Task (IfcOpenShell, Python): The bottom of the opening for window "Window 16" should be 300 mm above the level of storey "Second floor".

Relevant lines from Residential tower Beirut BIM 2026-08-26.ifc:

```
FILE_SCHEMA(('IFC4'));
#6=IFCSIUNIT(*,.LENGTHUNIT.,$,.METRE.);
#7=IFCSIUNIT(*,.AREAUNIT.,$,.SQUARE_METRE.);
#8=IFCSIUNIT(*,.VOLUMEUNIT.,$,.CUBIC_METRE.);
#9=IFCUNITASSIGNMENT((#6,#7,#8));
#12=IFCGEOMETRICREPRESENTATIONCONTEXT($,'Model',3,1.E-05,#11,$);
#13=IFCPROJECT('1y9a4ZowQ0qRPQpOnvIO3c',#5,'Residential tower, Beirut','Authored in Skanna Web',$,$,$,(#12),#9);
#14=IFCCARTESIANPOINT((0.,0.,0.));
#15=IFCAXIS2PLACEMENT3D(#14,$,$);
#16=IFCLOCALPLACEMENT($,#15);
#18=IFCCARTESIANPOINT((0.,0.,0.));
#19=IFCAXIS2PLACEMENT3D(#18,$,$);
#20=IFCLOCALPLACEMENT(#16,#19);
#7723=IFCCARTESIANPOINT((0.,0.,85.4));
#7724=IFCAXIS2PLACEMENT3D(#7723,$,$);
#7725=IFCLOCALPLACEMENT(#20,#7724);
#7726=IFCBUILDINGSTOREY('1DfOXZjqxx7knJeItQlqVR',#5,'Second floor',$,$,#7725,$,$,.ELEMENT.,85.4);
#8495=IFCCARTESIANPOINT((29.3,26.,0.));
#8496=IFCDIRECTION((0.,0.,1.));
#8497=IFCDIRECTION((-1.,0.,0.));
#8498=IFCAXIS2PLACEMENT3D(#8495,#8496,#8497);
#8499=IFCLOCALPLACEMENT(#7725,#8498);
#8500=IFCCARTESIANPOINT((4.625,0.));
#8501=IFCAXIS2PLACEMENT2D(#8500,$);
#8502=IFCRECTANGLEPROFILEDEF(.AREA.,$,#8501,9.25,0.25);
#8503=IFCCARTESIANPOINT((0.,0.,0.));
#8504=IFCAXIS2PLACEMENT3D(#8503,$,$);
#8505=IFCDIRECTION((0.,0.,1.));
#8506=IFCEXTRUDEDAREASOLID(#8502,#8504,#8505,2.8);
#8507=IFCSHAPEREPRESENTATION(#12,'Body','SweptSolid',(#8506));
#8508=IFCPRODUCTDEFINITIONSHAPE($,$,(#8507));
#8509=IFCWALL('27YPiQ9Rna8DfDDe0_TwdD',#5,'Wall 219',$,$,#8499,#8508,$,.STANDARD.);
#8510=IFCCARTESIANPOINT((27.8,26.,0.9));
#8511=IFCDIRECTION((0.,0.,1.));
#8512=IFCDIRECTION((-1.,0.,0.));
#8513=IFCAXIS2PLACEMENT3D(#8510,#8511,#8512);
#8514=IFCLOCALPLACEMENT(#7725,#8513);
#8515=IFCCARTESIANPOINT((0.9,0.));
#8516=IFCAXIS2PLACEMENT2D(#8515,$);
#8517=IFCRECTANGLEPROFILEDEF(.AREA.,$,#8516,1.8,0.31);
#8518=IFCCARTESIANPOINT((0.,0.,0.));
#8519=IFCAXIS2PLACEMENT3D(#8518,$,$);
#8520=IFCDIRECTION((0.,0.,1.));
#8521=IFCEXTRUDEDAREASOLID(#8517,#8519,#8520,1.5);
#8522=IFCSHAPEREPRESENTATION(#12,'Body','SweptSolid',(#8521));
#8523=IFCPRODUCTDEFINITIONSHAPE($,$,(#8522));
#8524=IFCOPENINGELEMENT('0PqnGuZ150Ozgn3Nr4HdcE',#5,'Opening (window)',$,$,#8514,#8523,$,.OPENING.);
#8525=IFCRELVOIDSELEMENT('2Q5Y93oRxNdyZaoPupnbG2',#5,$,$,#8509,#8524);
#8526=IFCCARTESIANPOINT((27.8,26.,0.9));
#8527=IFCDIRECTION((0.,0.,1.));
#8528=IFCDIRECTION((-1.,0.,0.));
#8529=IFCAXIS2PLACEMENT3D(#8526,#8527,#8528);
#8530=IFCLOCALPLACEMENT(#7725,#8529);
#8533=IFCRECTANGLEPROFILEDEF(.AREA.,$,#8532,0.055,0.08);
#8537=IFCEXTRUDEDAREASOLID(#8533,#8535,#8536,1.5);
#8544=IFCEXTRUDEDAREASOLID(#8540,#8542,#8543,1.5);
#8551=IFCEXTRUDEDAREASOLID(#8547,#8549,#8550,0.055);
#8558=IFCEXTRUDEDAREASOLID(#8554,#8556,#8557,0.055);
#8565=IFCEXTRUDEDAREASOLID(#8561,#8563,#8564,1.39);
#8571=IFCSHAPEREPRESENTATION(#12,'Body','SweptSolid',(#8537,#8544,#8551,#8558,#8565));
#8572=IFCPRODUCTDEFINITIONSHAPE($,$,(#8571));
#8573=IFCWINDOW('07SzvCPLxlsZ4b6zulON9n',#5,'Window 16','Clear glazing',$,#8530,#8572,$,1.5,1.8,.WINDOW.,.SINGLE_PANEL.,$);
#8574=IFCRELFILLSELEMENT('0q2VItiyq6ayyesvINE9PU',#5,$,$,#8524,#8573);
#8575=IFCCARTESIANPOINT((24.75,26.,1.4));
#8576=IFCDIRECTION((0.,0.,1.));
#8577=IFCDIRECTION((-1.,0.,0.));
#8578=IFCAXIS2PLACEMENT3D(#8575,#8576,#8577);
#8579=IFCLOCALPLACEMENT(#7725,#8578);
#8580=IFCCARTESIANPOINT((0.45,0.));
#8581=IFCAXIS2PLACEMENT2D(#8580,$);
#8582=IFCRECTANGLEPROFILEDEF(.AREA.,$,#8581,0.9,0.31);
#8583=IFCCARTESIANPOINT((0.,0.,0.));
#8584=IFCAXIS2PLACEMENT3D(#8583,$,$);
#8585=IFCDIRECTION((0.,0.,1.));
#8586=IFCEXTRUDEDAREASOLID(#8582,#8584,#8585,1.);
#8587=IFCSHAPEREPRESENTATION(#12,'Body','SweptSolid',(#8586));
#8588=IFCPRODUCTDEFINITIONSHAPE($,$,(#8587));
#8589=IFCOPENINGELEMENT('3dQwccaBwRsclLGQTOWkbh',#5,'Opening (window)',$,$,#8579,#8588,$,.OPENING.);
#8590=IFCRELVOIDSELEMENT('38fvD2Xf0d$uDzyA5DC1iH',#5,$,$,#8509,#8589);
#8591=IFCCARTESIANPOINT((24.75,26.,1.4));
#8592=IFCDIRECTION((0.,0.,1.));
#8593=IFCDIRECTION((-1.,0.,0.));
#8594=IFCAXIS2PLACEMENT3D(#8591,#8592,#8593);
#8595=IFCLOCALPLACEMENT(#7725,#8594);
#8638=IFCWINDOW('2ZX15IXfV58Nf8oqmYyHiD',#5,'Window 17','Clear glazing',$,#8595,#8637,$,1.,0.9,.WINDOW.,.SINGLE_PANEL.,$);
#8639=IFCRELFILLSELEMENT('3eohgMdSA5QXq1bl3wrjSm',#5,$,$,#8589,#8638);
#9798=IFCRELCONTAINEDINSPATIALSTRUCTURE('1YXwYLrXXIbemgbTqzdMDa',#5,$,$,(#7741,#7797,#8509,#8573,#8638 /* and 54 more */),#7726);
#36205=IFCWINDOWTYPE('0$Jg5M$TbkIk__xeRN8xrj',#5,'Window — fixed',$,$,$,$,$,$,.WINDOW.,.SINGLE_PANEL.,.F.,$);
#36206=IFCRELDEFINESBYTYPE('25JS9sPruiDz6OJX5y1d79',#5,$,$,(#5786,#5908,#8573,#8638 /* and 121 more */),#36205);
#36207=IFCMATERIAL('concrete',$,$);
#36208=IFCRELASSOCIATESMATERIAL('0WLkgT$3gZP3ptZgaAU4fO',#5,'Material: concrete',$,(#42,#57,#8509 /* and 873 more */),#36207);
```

```python
import numpy as np
import ifcopenshell
import ifcopenshell.api.geometry
import ifcopenshell.geom
import ifcopenshell.util.element
import ifcopenshell.util.placement
import ifcopenshell.util.shape
import ifcopenshell.util.unit

model = ifcopenshell.open("Residential tower Beirut BIM 2026-08-26.ifc")
unit_scale = ifcopenshell.util.unit.calculate_unit_scale(model)

window = model.by_guid("07SzvCPLxlsZ4b6zulON9n")
opening = window.FillsVoids[0].RelatingOpeningElement
storey = ifcopenshell.util.element.get_container(window, ifc_class="IfcBuildingStorey")
level = ifcopenshell.util.placement.get_local_placement(storey.ObjectPlacement)[2, 3]

# The opening's origin need not be at the sill, so measure its lowest point.
shape = ifcopenshell.geom.create_shape(ifcopenshell.geom.settings(), opening)
bottom = ifcopenshell.util.shape.get_shape_bottom_elevation(shape, shape.geometry) / unit_scale
dz = level + 0.3 / unit_scale - bottom

shift = np.array([0.0, 0.0, dz])
# The window is not placed relative to its opening, so move both.
for product in (opening, window):
    matrix = ifcopenshell.util.placement.get_local_placement(product.ObjectPlacement)
    matrix[:3, 3] += shift
    ifcopenshell.api.geometry.edit_object_placement(model, product=product, matrix=matrix, is_si=False)

print(f"moved by {dz * unit_scale:+.3f} m")

model.write("Residential tower Beirut BIM 2026-08-26_rev.ifc")
```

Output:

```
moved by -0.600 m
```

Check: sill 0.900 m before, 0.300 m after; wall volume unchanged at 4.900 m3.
